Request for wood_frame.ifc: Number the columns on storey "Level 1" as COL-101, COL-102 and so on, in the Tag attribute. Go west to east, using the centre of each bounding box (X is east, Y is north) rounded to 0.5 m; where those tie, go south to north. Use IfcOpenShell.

First a look at what the model holds.

```python
import ifcopenshell
import ifcopenshell.util.element
import ifcopenshell.util.placement

model = ifcopenshell.open("wood_frame.ifc")
print(model.schema)
storey = next(s for s in model.by_type("IfcBuildingStorey") if s.Name == "Level 1")
columns = [e for e in ifcopenshell.util.element.get_decomposition(storey) if e.is_a("IfcColumn")]
for e in sorted(columns, key=lambda e: e.id()):
    origin = ifcopenshell.util.placement.get_local_placement(e.ObjectPlacement)[:3, 3]
    print(e.id(), e.Tag, e.Name, origin.round(2) + 0.0, sep=" | ")
```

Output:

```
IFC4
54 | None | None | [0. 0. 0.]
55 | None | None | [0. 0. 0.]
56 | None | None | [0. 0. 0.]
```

```python
import ifcopenshell
import ifcopenshell.geom
import ifcopenshell.util.element
import ifcopenshell.util.shape

model = ifcopenshell.open("wood_frame.ifc")
settings = ifcopenshell.geom.settings()
settings.set("use-world-coords", True)


def centre(element):
    shape = ifcopenshell.geom.create_shape(settings, element)
    return ifcopenshell.util.shape.get_bbox_centroid(shape.geometry)


storey = next(s for s in model.by_type("IfcBuildingStorey") if s.Name == "Level 1")
columns = [e for e in ifcopenshell.util.element.get_decomposition(storey) if e.is_a("IfcColumn")]

# Insertion points can sit at a corner or the storey origin, so sort by the geometry (in metres).
centres = {e: centre(e) for e in columns}
columns.sort(key=lambda e: (round(centres[e][0] / 0.5), centres[e][1]))

for i, e in enumerate(columns, start=1):
    number = f"COL-1{i:02d}"
    e.Tag = number
    print(e.id(), number)

model.write("wood_frame_rev.ifc")
```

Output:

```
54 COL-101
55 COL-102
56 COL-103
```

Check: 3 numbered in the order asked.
